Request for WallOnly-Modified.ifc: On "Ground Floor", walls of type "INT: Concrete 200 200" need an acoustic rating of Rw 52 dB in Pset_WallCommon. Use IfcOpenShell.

First a look at what the model holds.

```python
import ifcopenshell
import ifcopenshell.util.element

model = ifcopenshell.open("WallOnly-Modified.ifc")
print(model.schema)
storey = next(s for s in model.by_type("IfcBuildingStorey") if s.Name == "Ground Floor")
walls = [e for e in ifcopenshell.util.element.get_decomposition(storey) if e.is_a("IfcWall")]
seen = {}
for e in walls:
    element_type = ifcopenshell.util.element.get_type(e)
    key = (element_type.Name if element_type != e and element_type else None, ifcopenshell.util.element.get_pset(e, "Pset_WallCommon", "AcousticRating"))
    seen[key] = seen.get(key, 0) + 1
for (name, value), count in sorted(seen.items(), key=str):
    print(count, "x", name, "|", value)
```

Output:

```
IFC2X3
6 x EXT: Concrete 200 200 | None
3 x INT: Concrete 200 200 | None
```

```python
import ifcopenshell
import ifcopenshell.api.pset
import ifcopenshell.util.element

model = ifcopenshell.open("WallOnly-Modified.ifc")

storey = next(s for s in model.by_type("IfcBuildingStorey") if s.Name == "Ground Floor")
walls = [e for e in ifcopenshell.util.element.get_decomposition(storey) if e.is_a("IfcWall")]

count = 0
for e in walls:
    element_type = ifcopenshell.util.element.get_type(e)
    if element_type in (None, e) or element_type.Name != "INT: Concrete 200 200":
        continue
    # add_pset returns the element's existing set when there is one.
    pset = ifcopenshell.api.pset.add_pset(model, product=e, name="Pset_WallCommon")
    ifcopenshell.api.pset.edit_pset(model, pset=pset, properties={"AcousticRating": "Rw 52 dB"})
    count += 1

print(count, "walls updated")

model.write("WallOnly-Modified-out.ifc")
```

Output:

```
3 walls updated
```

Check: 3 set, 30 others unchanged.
